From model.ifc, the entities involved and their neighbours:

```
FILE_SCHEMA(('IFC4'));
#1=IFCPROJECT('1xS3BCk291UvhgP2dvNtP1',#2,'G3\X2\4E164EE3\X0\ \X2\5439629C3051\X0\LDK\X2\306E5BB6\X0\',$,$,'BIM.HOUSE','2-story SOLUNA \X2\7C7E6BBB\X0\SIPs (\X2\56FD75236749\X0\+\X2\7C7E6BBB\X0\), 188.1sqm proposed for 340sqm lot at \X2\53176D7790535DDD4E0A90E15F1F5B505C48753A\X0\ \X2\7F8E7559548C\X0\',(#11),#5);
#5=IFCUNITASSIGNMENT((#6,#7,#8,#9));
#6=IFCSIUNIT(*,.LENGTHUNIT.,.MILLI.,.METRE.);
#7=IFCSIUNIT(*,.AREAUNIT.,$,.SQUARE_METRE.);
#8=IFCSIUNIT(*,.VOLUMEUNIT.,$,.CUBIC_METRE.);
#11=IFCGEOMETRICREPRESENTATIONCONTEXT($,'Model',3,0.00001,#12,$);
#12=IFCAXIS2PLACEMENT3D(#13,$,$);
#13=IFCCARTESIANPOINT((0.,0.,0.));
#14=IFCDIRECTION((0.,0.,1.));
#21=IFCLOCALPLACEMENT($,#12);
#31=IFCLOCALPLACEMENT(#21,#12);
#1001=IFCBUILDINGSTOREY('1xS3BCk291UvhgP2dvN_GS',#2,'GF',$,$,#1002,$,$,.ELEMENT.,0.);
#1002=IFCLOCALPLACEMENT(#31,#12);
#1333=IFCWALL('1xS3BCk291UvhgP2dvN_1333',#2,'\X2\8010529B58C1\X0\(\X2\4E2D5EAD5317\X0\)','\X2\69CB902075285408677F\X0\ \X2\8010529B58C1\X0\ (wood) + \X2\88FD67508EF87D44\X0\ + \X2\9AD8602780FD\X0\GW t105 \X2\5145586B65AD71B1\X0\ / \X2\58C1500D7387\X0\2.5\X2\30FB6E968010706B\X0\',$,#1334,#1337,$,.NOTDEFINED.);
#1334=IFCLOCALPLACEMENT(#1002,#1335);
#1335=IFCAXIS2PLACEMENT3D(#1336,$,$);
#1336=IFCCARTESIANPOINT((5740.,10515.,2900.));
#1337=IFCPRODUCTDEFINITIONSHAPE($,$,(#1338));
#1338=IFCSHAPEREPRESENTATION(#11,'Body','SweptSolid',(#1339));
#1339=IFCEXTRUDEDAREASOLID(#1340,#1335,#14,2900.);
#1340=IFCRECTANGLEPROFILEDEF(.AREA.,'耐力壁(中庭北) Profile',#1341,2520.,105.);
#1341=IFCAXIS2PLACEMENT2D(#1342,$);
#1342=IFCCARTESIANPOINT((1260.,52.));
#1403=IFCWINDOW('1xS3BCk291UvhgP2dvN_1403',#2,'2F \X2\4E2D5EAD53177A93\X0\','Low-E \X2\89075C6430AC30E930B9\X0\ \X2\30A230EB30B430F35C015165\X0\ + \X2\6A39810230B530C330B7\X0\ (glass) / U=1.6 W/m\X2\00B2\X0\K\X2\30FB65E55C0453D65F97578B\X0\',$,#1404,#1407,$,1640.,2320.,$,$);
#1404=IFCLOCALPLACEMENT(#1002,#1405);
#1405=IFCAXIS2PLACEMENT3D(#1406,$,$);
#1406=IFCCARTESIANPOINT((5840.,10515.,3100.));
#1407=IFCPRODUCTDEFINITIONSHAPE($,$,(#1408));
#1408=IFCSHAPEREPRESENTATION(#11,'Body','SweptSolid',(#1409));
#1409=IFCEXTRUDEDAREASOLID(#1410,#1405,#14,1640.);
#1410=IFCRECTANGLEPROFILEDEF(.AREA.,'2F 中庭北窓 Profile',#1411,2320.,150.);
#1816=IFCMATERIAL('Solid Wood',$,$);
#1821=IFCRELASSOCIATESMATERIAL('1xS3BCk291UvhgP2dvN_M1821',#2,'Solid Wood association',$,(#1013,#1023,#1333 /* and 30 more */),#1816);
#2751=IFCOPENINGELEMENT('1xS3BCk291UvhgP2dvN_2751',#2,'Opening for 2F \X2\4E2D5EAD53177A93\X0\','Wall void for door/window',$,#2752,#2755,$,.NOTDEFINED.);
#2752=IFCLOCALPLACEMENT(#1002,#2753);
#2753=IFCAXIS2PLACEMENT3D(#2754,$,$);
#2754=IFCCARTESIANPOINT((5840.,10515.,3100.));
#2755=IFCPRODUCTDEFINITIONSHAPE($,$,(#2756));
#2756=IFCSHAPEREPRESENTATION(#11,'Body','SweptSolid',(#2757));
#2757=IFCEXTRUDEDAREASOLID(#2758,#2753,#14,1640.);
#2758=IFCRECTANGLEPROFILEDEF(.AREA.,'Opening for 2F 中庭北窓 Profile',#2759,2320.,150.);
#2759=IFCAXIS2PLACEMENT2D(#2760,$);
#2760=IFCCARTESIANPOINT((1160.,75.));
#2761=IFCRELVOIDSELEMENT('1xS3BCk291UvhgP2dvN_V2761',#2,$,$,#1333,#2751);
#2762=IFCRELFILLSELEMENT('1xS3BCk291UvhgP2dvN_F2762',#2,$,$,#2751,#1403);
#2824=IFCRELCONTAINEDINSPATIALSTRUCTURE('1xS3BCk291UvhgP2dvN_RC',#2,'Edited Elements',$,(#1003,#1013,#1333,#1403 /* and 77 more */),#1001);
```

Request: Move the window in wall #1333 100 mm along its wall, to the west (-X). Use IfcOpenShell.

```python
import ifcopenshell
import ifcopenshell.api.geometry
import ifcopenshell.util.placement

model = ifcopenshell.open("model.ifc")

window = model.by_guid("1xS3BCk291UvhgP2dvN_1403")
opening = window.FillsVoids[0].RelatingOpeningElement
wall = opening.VoidsElements[0].RelatingBuildingElement

wall_matrix = ifcopenshell.util.placement.get_local_placement(wall.ObjectPlacement)
shift = wall_matrix[:3, 0] * -100.0
before = ifcopenshell.util.placement.get_local_placement(window.ObjectPlacement)[:3, 3].copy()

# The window is not placed relative to its opening, so move both.
for product in (opening, window):
    matrix = ifcopenshell.util.placement.get_local_placement(product.ObjectPlacement)
    matrix[:3, 3] += shift
    ifcopenshell.api.geometry.edit_object_placement(model, product=product, matrix=matrix, is_si=False)

after = ifcopenshell.util.placement.get_local_placement(window.ObjectPlacement)[:3, 3]
print("window moved by", (after - before).round(3) + 0.0)

model.write("model-out.ifc")
```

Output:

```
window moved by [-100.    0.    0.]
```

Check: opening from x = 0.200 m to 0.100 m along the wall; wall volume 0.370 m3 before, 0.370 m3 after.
